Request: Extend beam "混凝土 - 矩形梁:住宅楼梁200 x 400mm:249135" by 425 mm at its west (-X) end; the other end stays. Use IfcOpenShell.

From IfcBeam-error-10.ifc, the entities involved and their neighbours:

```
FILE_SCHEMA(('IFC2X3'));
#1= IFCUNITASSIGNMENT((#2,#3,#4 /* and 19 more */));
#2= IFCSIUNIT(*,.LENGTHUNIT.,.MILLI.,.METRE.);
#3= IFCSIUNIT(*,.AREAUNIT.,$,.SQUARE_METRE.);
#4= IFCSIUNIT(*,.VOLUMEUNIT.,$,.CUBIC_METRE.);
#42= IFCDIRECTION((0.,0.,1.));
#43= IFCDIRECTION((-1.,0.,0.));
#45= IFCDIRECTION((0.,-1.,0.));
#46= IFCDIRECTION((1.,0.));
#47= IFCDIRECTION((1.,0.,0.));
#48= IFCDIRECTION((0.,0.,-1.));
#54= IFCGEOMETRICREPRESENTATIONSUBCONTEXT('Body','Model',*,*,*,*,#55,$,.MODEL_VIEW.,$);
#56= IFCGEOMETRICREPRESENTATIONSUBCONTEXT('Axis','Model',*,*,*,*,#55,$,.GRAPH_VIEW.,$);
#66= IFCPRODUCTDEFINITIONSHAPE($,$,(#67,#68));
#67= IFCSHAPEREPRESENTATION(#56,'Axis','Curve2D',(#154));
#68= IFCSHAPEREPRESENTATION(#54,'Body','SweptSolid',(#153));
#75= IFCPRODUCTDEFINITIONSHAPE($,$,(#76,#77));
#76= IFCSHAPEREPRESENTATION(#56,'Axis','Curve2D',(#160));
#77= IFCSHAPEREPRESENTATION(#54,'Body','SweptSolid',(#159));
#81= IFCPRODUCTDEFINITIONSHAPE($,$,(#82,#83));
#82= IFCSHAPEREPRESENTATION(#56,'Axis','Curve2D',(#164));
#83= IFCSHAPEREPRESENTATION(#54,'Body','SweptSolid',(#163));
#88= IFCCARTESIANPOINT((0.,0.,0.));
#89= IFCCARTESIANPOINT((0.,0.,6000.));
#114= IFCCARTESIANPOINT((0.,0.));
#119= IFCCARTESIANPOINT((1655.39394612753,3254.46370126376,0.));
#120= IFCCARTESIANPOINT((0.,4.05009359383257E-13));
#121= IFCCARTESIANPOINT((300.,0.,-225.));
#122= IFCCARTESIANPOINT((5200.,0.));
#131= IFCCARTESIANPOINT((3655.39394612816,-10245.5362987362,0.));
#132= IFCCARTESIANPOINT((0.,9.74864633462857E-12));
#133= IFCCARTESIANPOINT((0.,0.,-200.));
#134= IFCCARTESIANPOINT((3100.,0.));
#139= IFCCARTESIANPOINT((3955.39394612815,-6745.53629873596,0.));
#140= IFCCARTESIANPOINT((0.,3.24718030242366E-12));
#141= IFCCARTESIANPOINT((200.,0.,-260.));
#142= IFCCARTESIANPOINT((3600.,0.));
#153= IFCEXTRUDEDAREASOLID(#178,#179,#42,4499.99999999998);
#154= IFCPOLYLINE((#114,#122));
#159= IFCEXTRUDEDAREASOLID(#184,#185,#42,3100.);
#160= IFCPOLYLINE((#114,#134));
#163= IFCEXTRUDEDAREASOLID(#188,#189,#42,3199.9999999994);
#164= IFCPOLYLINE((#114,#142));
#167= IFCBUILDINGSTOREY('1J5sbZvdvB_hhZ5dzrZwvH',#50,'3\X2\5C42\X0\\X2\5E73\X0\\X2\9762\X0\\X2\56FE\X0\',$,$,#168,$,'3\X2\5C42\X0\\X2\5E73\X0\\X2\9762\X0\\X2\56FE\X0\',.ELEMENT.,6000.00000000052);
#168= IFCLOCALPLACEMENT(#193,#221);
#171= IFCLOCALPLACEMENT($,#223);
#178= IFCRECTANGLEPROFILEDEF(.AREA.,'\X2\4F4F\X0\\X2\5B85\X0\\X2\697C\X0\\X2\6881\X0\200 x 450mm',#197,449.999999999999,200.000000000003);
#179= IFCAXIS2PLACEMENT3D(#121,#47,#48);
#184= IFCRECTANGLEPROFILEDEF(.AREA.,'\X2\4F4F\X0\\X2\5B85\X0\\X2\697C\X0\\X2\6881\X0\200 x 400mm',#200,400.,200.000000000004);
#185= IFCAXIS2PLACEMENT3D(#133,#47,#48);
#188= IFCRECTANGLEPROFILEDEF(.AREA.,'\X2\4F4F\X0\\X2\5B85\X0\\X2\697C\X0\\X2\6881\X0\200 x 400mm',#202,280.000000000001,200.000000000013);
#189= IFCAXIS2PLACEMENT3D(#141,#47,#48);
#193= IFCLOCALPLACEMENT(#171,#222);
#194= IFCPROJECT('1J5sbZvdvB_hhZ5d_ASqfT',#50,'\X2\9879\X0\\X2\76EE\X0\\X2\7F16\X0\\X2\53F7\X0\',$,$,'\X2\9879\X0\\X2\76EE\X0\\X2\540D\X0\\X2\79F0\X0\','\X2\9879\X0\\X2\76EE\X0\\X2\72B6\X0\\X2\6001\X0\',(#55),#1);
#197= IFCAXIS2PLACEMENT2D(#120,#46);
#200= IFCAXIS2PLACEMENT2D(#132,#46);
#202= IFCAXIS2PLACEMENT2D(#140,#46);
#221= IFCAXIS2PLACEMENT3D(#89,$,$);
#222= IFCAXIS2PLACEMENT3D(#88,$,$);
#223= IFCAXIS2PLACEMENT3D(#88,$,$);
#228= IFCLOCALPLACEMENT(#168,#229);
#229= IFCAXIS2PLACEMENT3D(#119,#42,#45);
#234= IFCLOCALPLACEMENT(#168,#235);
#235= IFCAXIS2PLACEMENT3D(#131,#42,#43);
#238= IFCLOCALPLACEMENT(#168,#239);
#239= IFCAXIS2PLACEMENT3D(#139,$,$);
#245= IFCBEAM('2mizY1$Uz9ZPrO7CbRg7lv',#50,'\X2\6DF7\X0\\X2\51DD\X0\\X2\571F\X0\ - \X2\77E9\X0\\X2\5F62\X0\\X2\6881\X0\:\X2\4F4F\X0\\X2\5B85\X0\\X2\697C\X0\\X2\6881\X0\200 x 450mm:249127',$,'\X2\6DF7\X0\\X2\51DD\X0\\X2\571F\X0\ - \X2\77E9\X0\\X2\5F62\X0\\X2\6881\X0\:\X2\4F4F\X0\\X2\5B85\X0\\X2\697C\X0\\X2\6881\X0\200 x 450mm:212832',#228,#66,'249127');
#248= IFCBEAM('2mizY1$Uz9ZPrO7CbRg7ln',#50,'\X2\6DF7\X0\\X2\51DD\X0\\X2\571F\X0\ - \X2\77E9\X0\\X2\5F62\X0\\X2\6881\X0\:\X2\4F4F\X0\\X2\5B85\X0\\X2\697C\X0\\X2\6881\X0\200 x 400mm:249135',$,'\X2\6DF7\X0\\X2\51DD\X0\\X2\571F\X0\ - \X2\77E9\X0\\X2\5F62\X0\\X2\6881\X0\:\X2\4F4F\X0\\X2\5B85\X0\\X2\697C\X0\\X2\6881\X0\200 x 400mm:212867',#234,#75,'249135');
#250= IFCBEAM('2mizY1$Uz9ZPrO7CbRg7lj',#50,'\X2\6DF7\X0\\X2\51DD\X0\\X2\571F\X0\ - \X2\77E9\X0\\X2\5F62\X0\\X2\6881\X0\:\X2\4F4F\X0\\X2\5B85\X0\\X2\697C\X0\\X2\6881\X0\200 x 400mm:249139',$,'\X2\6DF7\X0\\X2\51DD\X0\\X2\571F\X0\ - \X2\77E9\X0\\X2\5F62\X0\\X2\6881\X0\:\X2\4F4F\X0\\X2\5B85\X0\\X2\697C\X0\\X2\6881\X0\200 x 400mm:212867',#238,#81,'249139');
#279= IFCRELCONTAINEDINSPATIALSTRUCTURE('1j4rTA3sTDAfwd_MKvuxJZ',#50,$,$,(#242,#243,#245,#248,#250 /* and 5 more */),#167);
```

```python
import numpy as np
import ifcopenshell
import ifcopenshell.util.representation
import ifcopenshell.util.unit

model = ifcopenshell.open("IfcBeam-error-10.ifc")
unit_scale = ifcopenshell.util.unit.calculate_unit_scale(model)

member = model.by_guid("2mizY1$Uz9ZPrO7CbRg7ln")
change = 0.425 / unit_scale

# The extrusion runs towards the end named, so only its depth changes.
body = ifcopenshell.util.representation.get_representation(member, "Model", "Body")
solid = body.Items[0]
old_length = solid.Depth
solid.Depth += change

# Move the axis end point with it.
axis = next(r for r in member.Representation.Representations if r.RepresentationIdentifier == "Axis").Items[0]
start, end = (np.array(p.Coordinates) for p in axis.Points)
end = end + (end - start) / np.linalg.norm(end - start) * change
point = model.createIfcCartesianPoint(end.tolist())
axis.Points = [axis.Points[0], point]

print(f"length {old_length:g} -> {solid.Depth:g}")

model.write("IfcBeam-error-10_updated.ifc")
```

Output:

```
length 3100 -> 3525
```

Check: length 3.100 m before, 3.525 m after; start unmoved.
